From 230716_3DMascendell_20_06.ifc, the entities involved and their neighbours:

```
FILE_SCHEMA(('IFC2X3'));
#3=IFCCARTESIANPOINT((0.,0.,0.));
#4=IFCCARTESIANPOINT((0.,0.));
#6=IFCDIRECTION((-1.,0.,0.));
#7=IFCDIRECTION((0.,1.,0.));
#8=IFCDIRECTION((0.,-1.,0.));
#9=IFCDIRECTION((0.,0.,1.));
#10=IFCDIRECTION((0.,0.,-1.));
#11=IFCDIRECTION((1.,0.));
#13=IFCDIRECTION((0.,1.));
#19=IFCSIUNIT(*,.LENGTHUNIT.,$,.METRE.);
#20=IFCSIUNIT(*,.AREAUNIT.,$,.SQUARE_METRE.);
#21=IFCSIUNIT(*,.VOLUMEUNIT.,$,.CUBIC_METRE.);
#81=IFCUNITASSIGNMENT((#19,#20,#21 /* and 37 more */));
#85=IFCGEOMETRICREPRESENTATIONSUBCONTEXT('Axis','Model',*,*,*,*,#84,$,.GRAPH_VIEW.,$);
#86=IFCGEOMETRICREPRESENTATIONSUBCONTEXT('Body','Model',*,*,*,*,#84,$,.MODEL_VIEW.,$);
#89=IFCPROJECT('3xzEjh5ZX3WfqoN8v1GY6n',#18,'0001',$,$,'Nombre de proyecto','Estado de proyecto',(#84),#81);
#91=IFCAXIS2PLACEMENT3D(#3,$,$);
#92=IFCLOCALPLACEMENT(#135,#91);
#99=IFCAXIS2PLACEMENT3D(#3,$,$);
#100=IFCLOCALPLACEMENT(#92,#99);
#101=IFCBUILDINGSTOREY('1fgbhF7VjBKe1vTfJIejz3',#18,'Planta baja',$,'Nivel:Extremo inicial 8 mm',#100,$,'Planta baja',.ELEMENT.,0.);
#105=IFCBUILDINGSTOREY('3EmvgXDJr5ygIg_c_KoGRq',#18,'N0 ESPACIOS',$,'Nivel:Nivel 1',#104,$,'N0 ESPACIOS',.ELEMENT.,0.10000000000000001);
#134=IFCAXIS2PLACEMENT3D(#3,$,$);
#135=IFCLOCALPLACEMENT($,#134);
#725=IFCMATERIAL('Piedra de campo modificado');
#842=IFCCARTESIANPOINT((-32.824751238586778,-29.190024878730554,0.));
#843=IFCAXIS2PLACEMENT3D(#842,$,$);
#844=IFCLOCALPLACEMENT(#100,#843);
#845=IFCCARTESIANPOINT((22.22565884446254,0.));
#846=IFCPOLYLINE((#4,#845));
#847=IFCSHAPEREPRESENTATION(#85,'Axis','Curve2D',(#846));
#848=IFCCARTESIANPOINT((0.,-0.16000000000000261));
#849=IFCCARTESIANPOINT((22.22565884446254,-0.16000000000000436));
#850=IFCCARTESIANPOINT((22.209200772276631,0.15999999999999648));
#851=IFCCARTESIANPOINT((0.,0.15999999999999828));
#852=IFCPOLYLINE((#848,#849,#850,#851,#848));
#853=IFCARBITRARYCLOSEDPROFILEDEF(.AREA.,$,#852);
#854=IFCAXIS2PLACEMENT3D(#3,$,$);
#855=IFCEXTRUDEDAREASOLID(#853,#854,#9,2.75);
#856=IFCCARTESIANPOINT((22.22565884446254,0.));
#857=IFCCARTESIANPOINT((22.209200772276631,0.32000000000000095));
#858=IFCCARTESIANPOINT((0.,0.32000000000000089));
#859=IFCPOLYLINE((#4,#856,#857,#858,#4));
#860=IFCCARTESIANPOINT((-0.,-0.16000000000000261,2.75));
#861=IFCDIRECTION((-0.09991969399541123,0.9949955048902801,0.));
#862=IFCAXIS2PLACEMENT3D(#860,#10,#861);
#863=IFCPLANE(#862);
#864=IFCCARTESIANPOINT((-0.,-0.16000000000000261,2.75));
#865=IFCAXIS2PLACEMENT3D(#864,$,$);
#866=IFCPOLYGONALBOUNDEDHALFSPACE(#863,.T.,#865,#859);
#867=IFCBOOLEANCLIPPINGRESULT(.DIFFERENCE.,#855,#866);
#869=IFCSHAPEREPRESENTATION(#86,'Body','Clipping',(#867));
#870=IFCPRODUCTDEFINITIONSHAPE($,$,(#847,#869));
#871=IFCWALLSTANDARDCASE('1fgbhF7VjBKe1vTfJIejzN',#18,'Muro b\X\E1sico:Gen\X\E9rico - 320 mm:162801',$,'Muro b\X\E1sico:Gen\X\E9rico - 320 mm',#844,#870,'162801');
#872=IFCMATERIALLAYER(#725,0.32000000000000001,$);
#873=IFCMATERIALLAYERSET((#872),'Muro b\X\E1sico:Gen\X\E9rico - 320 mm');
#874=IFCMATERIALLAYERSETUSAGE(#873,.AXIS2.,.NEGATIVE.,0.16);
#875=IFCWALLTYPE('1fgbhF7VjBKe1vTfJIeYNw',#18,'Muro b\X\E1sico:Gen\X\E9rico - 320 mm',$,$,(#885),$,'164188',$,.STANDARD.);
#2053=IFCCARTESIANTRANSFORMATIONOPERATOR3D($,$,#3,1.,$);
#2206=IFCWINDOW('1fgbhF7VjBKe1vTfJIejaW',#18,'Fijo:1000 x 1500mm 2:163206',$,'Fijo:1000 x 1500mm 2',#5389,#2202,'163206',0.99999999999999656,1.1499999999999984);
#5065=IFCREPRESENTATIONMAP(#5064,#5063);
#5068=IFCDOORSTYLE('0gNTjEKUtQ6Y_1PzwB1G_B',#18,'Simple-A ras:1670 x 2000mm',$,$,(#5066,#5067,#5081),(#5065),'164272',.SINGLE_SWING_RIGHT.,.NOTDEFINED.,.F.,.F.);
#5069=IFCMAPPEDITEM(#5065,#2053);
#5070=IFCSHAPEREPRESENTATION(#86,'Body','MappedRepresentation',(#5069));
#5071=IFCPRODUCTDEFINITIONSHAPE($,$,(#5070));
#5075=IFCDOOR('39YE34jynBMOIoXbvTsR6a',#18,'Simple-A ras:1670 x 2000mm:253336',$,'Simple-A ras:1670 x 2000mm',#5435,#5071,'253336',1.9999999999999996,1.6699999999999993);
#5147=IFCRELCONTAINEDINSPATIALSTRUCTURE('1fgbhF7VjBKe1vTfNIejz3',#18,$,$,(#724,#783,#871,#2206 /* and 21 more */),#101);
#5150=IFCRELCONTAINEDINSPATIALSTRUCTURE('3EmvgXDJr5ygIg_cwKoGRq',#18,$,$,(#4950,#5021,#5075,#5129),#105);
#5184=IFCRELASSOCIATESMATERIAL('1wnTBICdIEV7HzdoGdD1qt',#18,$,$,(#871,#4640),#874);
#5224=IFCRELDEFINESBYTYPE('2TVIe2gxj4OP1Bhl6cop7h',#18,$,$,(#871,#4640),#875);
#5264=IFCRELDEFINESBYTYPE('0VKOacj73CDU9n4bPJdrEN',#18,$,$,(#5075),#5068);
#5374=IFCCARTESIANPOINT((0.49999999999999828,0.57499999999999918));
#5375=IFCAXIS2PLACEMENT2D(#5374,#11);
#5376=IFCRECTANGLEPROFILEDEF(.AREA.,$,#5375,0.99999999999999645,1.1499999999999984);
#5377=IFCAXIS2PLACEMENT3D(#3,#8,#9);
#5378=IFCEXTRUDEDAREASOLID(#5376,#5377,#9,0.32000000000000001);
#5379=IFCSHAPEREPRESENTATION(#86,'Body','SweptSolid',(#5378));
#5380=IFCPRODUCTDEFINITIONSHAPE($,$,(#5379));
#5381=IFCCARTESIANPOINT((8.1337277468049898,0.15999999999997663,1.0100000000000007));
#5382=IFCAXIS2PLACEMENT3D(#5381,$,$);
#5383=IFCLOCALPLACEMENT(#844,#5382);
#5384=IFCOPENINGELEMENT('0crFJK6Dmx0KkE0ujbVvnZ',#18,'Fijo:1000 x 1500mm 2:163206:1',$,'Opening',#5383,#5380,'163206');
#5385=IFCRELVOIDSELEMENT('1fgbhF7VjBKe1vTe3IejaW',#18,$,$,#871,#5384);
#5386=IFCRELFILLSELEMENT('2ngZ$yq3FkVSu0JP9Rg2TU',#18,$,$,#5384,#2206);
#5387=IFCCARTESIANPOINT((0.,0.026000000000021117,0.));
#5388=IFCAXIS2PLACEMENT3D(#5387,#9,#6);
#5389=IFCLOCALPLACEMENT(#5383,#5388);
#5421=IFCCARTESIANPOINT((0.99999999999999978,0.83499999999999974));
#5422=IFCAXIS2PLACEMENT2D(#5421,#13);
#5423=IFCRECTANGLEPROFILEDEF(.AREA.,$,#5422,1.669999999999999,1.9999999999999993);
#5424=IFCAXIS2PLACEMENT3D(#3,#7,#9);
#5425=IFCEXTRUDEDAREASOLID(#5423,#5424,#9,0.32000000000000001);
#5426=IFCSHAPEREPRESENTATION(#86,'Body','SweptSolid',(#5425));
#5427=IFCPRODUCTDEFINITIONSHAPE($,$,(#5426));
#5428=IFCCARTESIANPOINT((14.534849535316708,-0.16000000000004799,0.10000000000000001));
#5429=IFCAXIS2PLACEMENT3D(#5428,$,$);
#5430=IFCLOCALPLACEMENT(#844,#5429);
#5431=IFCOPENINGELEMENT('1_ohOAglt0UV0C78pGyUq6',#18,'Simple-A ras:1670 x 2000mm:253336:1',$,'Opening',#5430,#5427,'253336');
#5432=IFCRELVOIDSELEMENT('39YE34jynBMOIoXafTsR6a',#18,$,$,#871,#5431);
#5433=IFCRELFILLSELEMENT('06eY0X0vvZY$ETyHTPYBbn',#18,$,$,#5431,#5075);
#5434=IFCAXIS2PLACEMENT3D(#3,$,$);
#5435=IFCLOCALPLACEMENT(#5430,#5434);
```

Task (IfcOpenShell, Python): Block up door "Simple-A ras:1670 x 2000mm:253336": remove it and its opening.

```python
import ifcopenshell
import ifcopenshell.api.feature
import ifcopenshell.api.root
import ifcopenshell.geom
import ifcopenshell.util.shape

model = ifcopenshell.open("230716_3DMascendell_20_06.ifc")
settings = ifcopenshell.geom.settings()


def volume(element):
    """Net volume in cubic metres, openings subtracted."""
    shape = ifcopenshell.geom.create_shape(settings, element)
    return ifcopenshell.util.shape.get_volume(shape.geometry)


door = model.by_id(5075)
opening = door.FillsVoids[0].RelatingOpeningElement
wall = opening.VoidsElements[0].RelatingBuildingElement
before = volume(wall)

ifcopenshell.api.root.remove_product(model, product=door)
ifcopenshell.api.feature.remove_feature(model, feature=opening)

after = volume(wall)

print(f"wall volume {before:.3f} -> {after:.3f} m3")

model.write("230716_3DMascendell_20_06_rev.ifc")
```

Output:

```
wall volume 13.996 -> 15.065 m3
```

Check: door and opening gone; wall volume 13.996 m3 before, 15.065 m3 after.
